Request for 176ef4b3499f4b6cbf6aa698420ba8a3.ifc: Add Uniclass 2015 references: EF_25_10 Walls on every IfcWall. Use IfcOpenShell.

First a look at what the model holds.

```python
import ifcopenshell

model = ifcopenshell.open("176ef4b3499f4b6cbf6aa698420ba8a3.ifc")
print(model.schema)
print("classifications:", [c.Name for c in model.by_type("IfcClassification")])
for ifc_class in ("IfcDoor", "IfcRoof", "IfcStair", "IfcWall", "IfcWindow"):
    print(ifc_class, len(model.by_type(ifc_class)))
```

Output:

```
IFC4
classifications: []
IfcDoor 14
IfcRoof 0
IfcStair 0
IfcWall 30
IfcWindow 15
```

```python
import ifcopenshell
import ifcopenshell.api.classification

model = ifcopenshell.open("176ef4b3499f4b6cbf6aa698420ba8a3.ifc")

system = ifcopenshell.api.classification.add_classification(model, classification="Uniclass 2015")

codes = {
    "IfcWall": ("EF_25_10", "Walls"),
}
for ifc_class, (code, name) in codes.items():
    products = model.by_type(ifc_class)
    ifcopenshell.api.classification.add_reference(
        model, products=products, classification=system, identification=code, name=name
    )
    print(code, len(products))

model.write("176ef4b3499f4b6cbf6aa698420ba8a3-out.ifc")
```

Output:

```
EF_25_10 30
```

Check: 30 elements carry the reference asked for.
